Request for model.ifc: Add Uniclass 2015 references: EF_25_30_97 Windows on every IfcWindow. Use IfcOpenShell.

First a look at what the model holds.

```python
import ifcopenshell

model = ifcopenshell.open("model.ifc")
print(model.schema)
print("classifications:", [c.Name for c in model.by_type("IfcClassification")])
for ifc_class in ("IfcDoor", "IfcRoof", "IfcStair", "IfcWall", "IfcWindow"):
    print(ifc_class, len(model.by_type(ifc_class)))
```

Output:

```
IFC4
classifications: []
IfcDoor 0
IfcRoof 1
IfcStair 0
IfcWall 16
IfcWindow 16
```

```python
import ifcopenshell
import ifcopenshell.api.classification

model = ifcopenshell.open("model.ifc")

system = ifcopenshell.api.classification.add_classification(model, classification="Uniclass 2015")

codes = {
    "IfcWindow": ("EF_25_30_97", "Windows"),
}
for ifc_class, (code, name) in codes.items():
    products = model.by_type(ifc_class)
    ifcopenshell.api.classification.add_reference(
        model, products=products, classification=system, identification=code, name=name
    )
    print(code, len(products))

model.write("model-out.ifc")
```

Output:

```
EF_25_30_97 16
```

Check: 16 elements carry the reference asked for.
